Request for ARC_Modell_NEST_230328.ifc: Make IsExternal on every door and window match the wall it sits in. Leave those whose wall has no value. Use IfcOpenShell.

First a look at what the model holds.

```python
import ifcopenshell
import ifcopenshell.util.element

model = ifcopenshell.open("ARC_Modell_NEST_230328.ifc")
print(model.schema)
seen = {}
for e in model.by_type("IfcDoor") + model.by_type("IfcWindow"):
    if not e.FillsVoids:
        continue
    host = e.FillsVoids[0].RelatingOpeningElement.VoidsElements[0].RelatingBuildingElement
    own = ifcopenshell.util.element.get_pset(e, f"Pset_{e.is_a()[3:].removesuffix('StandardCase')}Common", "IsExternal")
    wall = ifcopenshell.util.element.get_pset(host, "Pset_WallCommon", "IsExternal")
    seen[e.is_a(), own, wall] = seen.get((e.is_a(), own, wall), 0) + 1
for (cls, own, wall), count in sorted(seen.items(), key=str):
    print(count, cls, "IsExternal:", own, "| host wall:", wall)
```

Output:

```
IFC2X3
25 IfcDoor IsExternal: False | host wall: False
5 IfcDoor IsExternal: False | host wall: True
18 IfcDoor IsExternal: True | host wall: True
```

```python
import ifcopenshell
import ifcopenshell.api.pset
import ifcopenshell.util.element

model = ifcopenshell.open("ARC_Modell_NEST_230328.ifc")

count = 0
for ifc_class, pset_name in (("IfcDoor", "Pset_DoorCommon"), ("IfcWindow", "Pset_WindowCommon")):
    for e in model.by_type(ifc_class):
        if not e.FillsVoids:
            continue
        host = e.FillsVoids[0].RelatingOpeningElement.VoidsElements[0].RelatingBuildingElement
        external = ifcopenshell.util.element.get_pset(host, "Pset_WallCommon", "IsExternal")
        if external is None or ifcopenshell.util.element.get_pset(e, pset_name, "IsExternal") == external:
            continue
        pset = ifcopenshell.api.pset.add_pset(model, product=e, name=pset_name)
        ifcopenshell.api.pset.edit_pset(model, pset=pset, properties={"IsExternal": external})
        count += 1

print(count, "updated")

model.write("ARC_Modell_NEST_230328-out.ifc")
```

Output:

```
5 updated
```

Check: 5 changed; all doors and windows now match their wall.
